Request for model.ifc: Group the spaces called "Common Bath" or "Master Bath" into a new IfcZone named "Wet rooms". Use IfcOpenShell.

First a look at what the model holds.

```python
import ifcopenshell

model = ifcopenshell.open("model.ifc")
print(model.schema)
seen = {}
for space in model.by_type("IfcSpace"):
    seen[space.LongName] = seen.get(space.LongName, 0) + 1
for name, count in sorted(seen.items(), key=str):
    print(count, "x", name)
print("zones:", [z.Name for z in model.by_type("IfcZone")][:20])
```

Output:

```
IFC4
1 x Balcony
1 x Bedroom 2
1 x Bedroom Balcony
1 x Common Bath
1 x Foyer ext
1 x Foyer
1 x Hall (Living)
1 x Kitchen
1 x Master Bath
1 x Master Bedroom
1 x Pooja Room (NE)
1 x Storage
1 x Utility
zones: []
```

```python
import ifcopenshell
import ifcopenshell.api.group
import ifcopenshell.api.root

model = ifcopenshell.open("model.ifc")

names = {"Common Bath", "Master Bath"}
spaces = [s for s in model.by_type("IfcSpace") if s.LongName in names]

zone = ifcopenshell.api.root.create_entity(model, ifc_class="IfcZone", name="Wet rooms")
ifcopenshell.api.group.assign_group(model, products=spaces, group=zone)
print(len(spaces), "spaces in", zone.Name)

model.write("model-out.ifc")
```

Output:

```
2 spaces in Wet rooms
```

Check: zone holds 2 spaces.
